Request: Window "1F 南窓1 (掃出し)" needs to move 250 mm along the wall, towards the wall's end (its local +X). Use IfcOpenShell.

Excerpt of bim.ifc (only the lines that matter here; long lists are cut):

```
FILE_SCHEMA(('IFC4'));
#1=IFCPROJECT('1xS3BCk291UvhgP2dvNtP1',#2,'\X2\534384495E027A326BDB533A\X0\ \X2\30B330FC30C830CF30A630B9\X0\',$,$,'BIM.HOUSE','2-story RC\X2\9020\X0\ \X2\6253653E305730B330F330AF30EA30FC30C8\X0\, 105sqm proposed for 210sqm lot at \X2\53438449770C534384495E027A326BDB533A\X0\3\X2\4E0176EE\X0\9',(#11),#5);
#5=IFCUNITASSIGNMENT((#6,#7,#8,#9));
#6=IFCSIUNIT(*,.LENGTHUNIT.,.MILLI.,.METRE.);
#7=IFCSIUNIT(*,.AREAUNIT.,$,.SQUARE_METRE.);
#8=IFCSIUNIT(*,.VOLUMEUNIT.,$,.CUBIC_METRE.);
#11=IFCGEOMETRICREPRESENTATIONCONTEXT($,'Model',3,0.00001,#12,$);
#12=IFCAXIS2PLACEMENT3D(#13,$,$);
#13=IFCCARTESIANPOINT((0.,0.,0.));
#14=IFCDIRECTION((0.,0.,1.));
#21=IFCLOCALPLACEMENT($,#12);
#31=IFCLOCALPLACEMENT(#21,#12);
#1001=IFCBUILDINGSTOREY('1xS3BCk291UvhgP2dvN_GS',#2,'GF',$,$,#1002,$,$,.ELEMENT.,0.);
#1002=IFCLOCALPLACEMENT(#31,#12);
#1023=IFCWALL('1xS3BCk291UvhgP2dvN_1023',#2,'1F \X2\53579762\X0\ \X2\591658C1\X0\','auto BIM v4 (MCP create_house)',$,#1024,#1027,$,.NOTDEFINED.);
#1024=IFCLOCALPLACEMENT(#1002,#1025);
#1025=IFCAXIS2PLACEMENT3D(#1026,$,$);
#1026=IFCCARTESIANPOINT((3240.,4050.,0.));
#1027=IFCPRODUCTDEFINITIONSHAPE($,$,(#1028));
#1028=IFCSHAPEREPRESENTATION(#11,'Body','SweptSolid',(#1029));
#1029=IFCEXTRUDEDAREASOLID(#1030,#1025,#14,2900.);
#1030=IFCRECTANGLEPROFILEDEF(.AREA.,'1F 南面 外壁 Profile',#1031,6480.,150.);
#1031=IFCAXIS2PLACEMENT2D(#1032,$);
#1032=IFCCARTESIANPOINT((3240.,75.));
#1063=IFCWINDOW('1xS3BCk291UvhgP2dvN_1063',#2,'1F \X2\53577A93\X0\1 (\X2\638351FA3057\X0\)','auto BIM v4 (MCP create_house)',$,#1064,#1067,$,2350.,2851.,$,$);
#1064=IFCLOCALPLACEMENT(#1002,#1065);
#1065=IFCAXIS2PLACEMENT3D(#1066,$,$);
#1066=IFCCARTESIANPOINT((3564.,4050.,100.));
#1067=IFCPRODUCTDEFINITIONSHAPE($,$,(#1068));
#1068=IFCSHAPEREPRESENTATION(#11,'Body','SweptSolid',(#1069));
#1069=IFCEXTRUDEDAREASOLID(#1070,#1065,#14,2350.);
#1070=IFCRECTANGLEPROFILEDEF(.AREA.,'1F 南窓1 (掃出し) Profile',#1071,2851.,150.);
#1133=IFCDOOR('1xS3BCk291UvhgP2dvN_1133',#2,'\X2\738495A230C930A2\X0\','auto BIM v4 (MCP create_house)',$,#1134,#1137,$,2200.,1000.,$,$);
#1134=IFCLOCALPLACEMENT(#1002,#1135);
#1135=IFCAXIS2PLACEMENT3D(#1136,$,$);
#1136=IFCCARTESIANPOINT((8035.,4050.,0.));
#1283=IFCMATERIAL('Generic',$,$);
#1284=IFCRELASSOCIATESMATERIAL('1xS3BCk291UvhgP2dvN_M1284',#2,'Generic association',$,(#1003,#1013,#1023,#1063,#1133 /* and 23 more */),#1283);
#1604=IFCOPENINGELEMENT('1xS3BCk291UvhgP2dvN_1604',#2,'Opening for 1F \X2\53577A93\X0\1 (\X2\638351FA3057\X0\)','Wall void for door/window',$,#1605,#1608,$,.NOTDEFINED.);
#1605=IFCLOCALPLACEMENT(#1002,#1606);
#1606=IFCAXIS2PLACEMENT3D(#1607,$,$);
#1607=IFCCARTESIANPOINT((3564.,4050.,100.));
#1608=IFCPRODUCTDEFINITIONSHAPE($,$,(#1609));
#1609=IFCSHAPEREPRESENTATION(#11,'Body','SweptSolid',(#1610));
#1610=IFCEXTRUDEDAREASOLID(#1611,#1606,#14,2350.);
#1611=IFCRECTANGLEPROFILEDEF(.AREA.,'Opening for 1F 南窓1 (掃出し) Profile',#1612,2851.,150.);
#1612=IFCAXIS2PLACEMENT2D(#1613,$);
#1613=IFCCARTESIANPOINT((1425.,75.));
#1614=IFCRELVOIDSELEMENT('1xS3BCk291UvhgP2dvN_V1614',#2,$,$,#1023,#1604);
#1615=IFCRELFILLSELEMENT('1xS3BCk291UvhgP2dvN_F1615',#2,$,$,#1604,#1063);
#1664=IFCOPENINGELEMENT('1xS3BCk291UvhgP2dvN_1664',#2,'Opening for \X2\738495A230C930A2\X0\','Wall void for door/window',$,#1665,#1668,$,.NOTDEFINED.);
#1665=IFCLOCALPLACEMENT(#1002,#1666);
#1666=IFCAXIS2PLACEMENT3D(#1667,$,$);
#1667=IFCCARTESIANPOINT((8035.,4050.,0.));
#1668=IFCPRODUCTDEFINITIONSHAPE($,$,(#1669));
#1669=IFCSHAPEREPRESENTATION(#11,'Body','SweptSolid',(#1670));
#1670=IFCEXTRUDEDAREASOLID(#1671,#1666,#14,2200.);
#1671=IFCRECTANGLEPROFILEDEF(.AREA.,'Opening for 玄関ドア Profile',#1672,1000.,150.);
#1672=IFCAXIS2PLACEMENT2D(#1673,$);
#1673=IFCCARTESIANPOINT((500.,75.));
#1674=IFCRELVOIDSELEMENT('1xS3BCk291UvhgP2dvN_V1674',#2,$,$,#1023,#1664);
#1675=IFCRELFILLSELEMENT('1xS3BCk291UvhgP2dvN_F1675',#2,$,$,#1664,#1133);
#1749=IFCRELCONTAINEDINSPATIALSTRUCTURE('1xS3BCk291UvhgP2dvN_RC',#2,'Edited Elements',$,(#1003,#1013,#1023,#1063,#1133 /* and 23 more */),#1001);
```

```python
import ifcopenshell
import ifcopenshell.api.geometry
import ifcopenshell.util.placement
import ifcopenshell.util.unit

model = ifcopenshell.open("bim.ifc")
unit_scale = ifcopenshell.util.unit.calculate_unit_scale(model)

window = model.by_guid("1xS3BCk291UvhgP2dvN_1063")
opening = window.FillsVoids[0].RelatingOpeningElement
wall = opening.VoidsElements[0].RelatingBuildingElement

wall_matrix = ifcopenshell.util.placement.get_local_placement(wall.ObjectPlacement)
shift = wall_matrix[:3, 0] * 0.25 / unit_scale
before = ifcopenshell.util.placement.get_local_placement(window.ObjectPlacement)[:3, 3].copy()

# The window is not placed relative to its opening, so move both.
for product in (opening, window):
    matrix = ifcopenshell.util.placement.get_local_placement(product.ObjectPlacement)
    matrix[:3, 3] += shift
    ifcopenshell.api.geometry.edit_object_placement(model, product=product, matrix=matrix, is_si=False)

after = ifcopenshell.util.placement.get_local_placement(window.ObjectPlacement)[:3, 3]
print("window moved by", (after - before).round(3) + 0.0)

model.write("bim-out.ifc")
```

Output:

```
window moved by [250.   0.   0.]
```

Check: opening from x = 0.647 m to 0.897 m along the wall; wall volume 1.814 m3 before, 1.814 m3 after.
